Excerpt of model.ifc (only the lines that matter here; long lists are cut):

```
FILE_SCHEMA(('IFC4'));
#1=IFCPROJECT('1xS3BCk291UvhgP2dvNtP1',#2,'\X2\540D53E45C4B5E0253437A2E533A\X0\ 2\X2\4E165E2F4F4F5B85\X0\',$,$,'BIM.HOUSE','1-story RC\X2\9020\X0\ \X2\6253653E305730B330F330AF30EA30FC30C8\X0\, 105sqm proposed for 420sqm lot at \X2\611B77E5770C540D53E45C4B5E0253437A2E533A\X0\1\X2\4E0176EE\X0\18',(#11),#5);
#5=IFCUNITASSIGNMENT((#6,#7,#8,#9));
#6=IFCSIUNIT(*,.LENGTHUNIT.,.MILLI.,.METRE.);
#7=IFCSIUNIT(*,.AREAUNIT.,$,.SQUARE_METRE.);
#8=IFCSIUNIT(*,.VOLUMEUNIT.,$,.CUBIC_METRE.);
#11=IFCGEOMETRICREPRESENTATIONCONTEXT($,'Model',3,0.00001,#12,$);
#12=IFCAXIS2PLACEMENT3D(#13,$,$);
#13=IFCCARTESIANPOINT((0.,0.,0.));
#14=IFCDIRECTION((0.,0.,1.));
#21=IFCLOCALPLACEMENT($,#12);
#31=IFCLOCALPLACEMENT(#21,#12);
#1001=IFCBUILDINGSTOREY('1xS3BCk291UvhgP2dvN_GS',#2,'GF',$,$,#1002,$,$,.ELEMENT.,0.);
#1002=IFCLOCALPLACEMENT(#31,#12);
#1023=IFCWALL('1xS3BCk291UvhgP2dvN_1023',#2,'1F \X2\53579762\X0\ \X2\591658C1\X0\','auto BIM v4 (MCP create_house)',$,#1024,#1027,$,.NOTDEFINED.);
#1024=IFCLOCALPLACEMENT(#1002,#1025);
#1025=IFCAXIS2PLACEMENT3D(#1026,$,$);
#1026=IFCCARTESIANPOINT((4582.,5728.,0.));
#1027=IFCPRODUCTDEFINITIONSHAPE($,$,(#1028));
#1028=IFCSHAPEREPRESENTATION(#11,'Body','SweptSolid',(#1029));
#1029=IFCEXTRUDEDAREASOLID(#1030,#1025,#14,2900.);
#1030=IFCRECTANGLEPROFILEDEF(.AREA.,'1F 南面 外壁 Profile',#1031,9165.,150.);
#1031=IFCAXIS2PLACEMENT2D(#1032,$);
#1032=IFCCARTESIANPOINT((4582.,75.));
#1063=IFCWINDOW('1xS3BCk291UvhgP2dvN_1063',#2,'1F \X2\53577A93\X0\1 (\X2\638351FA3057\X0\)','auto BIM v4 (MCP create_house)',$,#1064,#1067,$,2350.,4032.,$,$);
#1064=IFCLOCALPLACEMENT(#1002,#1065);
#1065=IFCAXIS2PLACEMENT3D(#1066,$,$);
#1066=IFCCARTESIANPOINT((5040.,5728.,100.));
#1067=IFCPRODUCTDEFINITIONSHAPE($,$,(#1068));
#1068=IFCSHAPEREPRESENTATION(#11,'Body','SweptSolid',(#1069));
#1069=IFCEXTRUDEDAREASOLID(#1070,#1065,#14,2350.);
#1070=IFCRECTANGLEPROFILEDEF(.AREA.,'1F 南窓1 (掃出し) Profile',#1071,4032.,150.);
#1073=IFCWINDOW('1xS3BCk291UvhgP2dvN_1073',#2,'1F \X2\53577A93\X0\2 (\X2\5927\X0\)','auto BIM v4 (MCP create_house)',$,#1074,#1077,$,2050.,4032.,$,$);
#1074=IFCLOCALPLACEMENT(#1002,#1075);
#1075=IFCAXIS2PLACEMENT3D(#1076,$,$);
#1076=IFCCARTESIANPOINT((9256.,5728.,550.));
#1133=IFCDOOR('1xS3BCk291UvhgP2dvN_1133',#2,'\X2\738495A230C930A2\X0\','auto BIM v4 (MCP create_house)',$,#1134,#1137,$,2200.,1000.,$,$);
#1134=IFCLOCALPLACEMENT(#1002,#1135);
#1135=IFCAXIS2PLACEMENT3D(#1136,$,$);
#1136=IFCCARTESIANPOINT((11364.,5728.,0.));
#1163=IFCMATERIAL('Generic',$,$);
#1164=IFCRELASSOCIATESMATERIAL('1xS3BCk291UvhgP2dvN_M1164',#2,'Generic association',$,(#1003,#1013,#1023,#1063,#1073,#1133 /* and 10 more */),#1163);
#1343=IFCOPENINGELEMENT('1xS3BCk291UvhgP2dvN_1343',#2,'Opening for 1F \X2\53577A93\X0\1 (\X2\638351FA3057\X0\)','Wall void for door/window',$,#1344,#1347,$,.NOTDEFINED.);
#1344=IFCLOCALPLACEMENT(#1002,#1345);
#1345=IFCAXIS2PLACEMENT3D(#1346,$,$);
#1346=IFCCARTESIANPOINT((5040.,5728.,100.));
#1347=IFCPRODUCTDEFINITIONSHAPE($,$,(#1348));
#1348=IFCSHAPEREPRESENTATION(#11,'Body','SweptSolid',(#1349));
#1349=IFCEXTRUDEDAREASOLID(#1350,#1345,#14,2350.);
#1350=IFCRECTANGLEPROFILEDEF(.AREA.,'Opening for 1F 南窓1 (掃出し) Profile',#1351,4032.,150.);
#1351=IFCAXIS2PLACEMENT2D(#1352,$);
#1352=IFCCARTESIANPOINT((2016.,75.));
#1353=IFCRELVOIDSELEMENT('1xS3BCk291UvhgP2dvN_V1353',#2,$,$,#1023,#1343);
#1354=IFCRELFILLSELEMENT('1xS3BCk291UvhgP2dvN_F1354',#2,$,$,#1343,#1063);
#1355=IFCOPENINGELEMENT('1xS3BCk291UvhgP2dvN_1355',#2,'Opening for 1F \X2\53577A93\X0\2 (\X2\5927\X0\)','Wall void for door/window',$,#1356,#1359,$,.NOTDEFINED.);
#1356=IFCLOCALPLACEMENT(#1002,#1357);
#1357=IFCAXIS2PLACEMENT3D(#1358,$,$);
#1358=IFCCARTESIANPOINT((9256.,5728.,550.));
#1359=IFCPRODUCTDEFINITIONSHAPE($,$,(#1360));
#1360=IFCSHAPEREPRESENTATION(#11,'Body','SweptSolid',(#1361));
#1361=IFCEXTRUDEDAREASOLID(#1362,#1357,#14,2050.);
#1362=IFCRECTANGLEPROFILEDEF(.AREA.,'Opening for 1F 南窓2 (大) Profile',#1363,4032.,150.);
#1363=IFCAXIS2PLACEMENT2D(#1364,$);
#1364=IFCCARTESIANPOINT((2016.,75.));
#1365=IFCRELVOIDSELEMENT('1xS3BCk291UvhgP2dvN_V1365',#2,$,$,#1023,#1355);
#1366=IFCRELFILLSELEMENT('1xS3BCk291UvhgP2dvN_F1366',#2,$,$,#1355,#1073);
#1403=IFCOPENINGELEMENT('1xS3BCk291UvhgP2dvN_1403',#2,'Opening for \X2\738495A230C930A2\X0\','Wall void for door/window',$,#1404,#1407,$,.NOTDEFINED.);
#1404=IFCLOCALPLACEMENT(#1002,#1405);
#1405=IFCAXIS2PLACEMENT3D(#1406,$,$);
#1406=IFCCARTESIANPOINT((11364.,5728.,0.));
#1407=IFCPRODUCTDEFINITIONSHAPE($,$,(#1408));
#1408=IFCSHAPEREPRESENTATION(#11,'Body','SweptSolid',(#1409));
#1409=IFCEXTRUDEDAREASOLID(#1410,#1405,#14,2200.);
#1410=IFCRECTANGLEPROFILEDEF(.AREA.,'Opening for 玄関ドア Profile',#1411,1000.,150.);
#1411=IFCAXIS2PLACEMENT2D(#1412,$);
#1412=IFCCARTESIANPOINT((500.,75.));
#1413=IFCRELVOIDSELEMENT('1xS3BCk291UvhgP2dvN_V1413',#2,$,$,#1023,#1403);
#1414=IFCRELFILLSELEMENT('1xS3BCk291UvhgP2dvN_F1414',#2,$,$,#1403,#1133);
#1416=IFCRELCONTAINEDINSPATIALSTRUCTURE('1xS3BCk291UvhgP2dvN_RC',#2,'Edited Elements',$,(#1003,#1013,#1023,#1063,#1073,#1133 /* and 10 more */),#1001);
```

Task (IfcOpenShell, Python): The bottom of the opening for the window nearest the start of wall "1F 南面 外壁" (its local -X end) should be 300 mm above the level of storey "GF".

```python
import numpy as np
import ifcopenshell
import ifcopenshell.api.geometry
import ifcopenshell.geom
import ifcopenshell.util.element
import ifcopenshell.util.placement
import ifcopenshell.util.shape
import ifcopenshell.util.unit

model = ifcopenshell.open("model.ifc")
unit_scale = ifcopenshell.util.unit.calculate_unit_scale(model)

window = model.by_guid("1xS3BCk291UvhgP2dvN_1063")
opening = window.FillsVoids[0].RelatingOpeningElement
storey = ifcopenshell.util.element.get_container(window, ifc_class="IfcBuildingStorey")
level = ifcopenshell.util.placement.get_local_placement(storey.ObjectPlacement)[2, 3]

# The opening's origin need not be at the sill, so measure its lowest point.
shape = ifcopenshell.geom.create_shape(ifcopenshell.geom.settings(), opening)
bottom = ifcopenshell.util.shape.get_shape_bottom_elevation(shape, shape.geometry) / unit_scale
dz = level + 300.0 - bottom

shift = np.array([0.0, 0.0, dz])
# The window is not placed relative to its opening, so move both.
for product in (opening, window):
    matrix = ifcopenshell.util.placement.get_local_placement(product.ObjectPlacement)
    matrix[:3, 3] += shift
    ifcopenshell.api.geometry.edit_object_placement(model, product=product, matrix=matrix, is_si=False)

print(f"moved by {dz * unit_scale:+.3f} m")

model.write("model_updated.ifc")
```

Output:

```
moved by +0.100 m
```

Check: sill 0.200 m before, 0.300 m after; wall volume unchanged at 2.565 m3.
